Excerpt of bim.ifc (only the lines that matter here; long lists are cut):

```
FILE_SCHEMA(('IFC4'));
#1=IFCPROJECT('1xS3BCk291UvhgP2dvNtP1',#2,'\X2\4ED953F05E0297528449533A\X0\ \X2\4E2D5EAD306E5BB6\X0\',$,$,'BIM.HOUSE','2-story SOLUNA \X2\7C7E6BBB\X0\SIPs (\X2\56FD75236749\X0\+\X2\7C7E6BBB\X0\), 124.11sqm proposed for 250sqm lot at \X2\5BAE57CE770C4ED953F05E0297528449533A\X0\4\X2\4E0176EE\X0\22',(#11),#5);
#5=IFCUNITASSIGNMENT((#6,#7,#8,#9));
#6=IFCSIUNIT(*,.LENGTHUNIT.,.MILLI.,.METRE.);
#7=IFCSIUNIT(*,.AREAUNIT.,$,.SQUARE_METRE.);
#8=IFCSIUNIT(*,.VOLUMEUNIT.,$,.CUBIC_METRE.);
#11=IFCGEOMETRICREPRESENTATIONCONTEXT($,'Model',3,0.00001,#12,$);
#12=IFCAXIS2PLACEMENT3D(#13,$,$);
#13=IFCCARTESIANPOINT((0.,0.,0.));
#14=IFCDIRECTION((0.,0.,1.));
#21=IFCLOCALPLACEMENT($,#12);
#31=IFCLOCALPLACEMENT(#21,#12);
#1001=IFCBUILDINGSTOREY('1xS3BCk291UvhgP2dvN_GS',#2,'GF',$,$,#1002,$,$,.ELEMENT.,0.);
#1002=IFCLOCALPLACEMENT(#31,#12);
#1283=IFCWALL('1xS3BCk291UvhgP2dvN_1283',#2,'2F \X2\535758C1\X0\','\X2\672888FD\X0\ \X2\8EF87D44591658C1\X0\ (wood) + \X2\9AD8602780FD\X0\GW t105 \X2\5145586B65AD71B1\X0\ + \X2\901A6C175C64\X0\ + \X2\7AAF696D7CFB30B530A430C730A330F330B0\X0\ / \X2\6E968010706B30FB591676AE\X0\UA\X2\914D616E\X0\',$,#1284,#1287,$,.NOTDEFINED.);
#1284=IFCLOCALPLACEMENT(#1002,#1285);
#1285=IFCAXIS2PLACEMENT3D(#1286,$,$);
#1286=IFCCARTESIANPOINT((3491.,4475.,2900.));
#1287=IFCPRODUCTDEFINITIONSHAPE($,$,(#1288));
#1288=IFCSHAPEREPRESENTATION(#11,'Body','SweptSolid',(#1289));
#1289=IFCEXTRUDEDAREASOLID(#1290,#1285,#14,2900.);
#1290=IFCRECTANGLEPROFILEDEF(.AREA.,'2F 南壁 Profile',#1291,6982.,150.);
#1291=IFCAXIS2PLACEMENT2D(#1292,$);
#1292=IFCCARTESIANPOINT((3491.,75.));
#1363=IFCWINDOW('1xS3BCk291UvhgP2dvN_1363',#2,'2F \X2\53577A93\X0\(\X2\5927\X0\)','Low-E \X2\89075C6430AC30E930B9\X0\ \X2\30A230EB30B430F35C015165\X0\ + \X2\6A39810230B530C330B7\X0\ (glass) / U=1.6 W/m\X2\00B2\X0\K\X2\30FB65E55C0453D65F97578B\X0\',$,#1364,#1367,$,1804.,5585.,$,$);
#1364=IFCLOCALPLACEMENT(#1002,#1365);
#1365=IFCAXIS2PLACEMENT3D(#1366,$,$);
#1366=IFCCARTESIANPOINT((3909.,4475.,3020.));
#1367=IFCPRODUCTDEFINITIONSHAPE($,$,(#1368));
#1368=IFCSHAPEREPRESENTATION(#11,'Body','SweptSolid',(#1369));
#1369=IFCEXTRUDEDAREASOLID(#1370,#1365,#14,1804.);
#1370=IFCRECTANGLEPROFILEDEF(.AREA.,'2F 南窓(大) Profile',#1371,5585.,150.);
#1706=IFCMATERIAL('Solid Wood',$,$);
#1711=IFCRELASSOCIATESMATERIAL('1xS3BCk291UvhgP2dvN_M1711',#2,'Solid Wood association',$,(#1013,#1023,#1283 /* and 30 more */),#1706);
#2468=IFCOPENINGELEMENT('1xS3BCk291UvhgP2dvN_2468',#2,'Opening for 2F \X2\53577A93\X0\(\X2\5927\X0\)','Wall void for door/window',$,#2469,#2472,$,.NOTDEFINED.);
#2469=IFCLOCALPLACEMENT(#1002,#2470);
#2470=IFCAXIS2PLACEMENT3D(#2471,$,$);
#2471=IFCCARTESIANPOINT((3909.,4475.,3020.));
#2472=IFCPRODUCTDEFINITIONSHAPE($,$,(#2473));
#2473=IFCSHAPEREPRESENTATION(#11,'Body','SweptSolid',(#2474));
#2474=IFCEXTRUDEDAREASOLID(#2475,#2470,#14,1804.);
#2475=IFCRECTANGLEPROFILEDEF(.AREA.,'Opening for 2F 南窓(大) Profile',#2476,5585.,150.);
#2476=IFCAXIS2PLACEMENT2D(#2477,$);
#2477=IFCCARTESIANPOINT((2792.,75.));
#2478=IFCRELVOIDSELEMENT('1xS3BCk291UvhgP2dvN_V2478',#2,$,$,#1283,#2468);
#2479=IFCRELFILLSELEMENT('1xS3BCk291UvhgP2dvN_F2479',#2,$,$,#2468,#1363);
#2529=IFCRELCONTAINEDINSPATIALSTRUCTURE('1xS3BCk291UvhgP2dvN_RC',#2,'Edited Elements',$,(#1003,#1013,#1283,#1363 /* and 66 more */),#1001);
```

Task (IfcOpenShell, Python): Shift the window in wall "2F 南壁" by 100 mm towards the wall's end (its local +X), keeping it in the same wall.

```python
import ifcopenshell
import ifcopenshell.api.geometry
import ifcopenshell.util.placement
import ifcopenshell.util.unit

model = ifcopenshell.open("bim.ifc")
unit_scale = ifcopenshell.util.unit.calculate_unit_scale(model)

window = model.by_guid("1xS3BCk291UvhgP2dvN_1363")
opening = window.FillsVoids[0].RelatingOpeningElement
wall = opening.VoidsElements[0].RelatingBuildingElement

wall_matrix = ifcopenshell.util.placement.get_local_placement(wall.ObjectPlacement)
shift = wall_matrix[:3, 0] * 0.1 / unit_scale
before = ifcopenshell.util.placement.get_local_placement(window.ObjectPlacement)[:3, 3].copy()

# The window is not placed relative to its opening, so move both.
for product in (opening, window):
    matrix = ifcopenshell.util.placement.get_local_placement(product.ObjectPlacement)
    matrix[:3, 3] += shift
    ifcopenshell.api.geometry.edit_object_placement(model, product=product, matrix=matrix, is_si=False)

after = ifcopenshell.util.placement.get_local_placement(window.ObjectPlacement)[:3, 3]
print("window moved by", (after - before).round(3) + 0.0)

model.write("bim_v2.ifc")
```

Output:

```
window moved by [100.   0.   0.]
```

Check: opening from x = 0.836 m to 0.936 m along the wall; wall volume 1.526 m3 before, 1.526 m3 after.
